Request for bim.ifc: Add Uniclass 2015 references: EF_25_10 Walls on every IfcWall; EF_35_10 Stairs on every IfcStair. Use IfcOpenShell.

First a look at what the model holds.

```python
import ifcopenshell

model = ifcopenshell.open("bim.ifc")
print(model.schema)
print("classifications:", [c.Name for c in model.by_type("IfcClassification")])
for ifc_class in ("IfcDoor", "IfcRoof", "IfcStair", "IfcWall", "IfcWindow"):
    print(ifc_class, len(model.by_type(ifc_class)))
```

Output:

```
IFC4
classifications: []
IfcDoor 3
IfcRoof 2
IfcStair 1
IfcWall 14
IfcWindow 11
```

```python
import ifcopenshell
import ifcopenshell.api.classification

model = ifcopenshell.open("bim.ifc")

system = ifcopenshell.api.classification.add_classification(model, classification="Uniclass 2015")

codes = {
    "IfcWall": ("EF_25_10", "Walls"),
    "IfcStair": ("EF_35_10", "Stairs"),
}
for ifc_class, (code, name) in codes.items():
    products = model.by_type(ifc_class)
    ifcopenshell.api.classification.add_reference(
        model, products=products, classification=system, identification=code, name=name
    )
    print(code, len(products))

model.write("bim_rev.ifc")
```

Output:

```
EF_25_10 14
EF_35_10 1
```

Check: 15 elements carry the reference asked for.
